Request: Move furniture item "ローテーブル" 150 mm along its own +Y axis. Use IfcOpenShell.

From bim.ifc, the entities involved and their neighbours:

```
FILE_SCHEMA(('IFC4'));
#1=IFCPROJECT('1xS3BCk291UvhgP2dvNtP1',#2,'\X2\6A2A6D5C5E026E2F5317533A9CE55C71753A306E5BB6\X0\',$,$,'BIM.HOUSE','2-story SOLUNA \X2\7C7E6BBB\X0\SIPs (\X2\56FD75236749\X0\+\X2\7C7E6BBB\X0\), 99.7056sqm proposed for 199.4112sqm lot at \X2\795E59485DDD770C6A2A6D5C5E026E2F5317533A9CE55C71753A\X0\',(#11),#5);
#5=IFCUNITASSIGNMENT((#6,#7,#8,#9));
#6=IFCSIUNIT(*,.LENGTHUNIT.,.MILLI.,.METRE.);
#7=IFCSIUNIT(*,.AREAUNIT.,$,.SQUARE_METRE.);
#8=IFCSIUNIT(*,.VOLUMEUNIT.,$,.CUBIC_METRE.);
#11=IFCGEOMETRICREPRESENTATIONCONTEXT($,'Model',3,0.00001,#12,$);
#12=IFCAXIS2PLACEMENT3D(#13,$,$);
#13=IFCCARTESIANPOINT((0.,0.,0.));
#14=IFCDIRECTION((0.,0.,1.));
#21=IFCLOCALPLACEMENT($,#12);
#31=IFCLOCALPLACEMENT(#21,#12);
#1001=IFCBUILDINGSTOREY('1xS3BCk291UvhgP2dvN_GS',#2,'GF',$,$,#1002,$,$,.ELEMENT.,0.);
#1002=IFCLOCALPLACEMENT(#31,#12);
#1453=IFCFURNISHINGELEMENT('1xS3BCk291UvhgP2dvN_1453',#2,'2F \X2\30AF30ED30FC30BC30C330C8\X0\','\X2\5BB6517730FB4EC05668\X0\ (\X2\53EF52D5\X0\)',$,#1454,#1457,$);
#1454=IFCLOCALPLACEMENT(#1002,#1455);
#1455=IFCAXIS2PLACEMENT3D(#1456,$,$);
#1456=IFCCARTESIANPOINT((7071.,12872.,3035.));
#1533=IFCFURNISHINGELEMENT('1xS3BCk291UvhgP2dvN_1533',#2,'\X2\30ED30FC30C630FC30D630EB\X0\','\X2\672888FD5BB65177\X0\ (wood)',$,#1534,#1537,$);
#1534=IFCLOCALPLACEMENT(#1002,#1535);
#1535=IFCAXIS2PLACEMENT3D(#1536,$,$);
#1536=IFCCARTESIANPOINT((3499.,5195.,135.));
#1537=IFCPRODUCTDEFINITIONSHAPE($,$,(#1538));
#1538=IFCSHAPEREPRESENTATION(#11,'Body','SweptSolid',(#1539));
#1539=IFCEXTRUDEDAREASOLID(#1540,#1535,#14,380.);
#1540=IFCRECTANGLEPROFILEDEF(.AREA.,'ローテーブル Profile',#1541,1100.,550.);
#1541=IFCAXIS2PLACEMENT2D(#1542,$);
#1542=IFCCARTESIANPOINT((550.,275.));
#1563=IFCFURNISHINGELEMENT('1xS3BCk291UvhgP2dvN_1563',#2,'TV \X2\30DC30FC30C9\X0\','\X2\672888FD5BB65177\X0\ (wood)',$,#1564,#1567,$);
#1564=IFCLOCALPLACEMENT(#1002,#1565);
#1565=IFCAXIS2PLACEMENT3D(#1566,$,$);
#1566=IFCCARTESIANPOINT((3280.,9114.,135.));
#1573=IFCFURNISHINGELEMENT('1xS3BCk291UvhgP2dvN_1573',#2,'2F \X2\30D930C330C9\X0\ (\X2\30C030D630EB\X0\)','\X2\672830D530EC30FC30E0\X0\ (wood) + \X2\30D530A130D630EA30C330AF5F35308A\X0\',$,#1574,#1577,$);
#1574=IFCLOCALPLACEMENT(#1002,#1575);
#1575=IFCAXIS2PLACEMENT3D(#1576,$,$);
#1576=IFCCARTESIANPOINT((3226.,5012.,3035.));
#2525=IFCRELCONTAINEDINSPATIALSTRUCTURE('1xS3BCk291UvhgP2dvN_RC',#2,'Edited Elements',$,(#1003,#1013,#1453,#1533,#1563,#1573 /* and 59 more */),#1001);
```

```python
import ifcopenshell
import ifcopenshell.api.geometry
import ifcopenshell.util.placement

model = ifcopenshell.open("bim.ifc")

item = model.by_id(1533)
matrix = ifcopenshell.util.placement.get_local_placement(item.ObjectPlacement)
matrix[:3, 3] += matrix[:3, 1] * 150.0
ifcopenshell.api.geometry.edit_object_placement(model, product=item, matrix=matrix, is_si=False)

print(ifcopenshell.util.placement.get_local_placement(item.ObjectPlacement).round(3) + 0.0)

model.write("bim_rev.ifc")
```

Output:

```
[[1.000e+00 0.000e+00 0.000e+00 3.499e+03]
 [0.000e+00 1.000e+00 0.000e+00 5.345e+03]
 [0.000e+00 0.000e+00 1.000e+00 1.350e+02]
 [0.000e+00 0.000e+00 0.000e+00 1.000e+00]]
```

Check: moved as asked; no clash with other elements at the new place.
